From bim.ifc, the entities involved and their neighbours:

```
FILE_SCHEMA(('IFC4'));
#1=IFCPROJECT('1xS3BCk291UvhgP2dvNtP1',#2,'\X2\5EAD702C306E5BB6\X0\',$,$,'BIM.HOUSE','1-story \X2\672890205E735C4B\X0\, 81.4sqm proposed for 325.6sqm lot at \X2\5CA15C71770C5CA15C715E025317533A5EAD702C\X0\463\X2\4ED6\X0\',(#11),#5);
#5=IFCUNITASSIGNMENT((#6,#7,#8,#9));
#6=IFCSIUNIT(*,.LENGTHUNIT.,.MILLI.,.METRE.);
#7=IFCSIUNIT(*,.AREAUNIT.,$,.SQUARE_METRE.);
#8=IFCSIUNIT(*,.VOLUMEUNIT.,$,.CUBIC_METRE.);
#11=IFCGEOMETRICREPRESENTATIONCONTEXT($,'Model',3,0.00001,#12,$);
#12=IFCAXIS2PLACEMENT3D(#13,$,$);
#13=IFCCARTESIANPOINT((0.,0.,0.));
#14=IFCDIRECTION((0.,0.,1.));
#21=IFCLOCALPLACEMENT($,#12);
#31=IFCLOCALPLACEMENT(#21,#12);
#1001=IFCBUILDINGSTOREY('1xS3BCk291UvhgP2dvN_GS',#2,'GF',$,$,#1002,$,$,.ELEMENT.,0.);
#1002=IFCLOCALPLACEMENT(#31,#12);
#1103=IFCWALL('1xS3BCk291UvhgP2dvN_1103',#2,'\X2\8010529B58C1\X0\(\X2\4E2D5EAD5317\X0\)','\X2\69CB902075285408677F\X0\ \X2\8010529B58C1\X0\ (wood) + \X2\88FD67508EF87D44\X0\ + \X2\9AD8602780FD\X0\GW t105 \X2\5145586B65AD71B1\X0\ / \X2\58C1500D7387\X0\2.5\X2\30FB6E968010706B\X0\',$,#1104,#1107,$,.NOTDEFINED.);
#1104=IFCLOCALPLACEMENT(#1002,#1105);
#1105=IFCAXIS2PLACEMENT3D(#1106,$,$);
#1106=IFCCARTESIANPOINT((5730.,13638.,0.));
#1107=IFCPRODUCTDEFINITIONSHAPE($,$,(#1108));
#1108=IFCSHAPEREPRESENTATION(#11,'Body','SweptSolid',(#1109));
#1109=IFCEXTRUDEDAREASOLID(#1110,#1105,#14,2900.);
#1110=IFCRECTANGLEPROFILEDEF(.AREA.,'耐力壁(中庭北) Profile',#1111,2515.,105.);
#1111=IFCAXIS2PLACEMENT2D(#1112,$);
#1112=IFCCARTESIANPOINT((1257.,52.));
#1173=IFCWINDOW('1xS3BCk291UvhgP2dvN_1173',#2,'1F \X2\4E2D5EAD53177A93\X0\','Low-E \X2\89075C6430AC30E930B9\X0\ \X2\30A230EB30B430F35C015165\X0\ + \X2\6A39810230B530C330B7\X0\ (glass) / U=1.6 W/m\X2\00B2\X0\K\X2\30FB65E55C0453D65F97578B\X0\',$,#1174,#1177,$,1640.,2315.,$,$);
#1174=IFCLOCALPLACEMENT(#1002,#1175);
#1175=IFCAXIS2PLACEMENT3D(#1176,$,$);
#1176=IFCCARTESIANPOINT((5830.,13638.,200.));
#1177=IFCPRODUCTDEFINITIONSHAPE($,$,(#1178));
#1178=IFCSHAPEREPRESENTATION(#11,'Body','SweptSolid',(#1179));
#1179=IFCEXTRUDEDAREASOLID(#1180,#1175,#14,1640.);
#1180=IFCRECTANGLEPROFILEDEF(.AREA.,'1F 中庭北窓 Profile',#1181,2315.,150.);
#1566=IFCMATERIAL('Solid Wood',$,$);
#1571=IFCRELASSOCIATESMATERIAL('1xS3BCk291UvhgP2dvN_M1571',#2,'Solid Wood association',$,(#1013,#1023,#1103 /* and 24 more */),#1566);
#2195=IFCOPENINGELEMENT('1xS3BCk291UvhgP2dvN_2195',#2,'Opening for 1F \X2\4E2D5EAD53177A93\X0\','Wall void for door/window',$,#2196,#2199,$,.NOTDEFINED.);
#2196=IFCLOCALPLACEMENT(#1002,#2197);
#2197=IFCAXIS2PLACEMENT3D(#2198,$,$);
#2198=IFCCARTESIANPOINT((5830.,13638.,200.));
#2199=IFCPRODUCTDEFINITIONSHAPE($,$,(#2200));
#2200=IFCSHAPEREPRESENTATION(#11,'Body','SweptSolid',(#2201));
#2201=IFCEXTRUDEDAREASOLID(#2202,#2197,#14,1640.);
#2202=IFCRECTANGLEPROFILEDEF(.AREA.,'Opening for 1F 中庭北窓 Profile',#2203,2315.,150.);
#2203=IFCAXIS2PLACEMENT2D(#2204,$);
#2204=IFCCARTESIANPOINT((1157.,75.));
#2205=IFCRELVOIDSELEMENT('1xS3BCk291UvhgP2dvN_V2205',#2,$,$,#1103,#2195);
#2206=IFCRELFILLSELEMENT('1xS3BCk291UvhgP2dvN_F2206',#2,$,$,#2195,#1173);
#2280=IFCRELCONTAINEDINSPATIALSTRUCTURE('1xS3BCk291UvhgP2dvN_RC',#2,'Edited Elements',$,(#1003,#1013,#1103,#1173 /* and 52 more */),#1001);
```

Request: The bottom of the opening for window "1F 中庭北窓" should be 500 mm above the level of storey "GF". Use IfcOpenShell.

```python
import numpy as np
import ifcopenshell
import ifcopenshell.api.geometry
import ifcopenshell.geom
import ifcopenshell.util.element
import ifcopenshell.util.placement
import ifcopenshell.util.shape
import ifcopenshell.util.unit

model = ifcopenshell.open("bim.ifc")
unit_scale = ifcopenshell.util.unit.calculate_unit_scale(model)

window = model.by_id(1173)
opening = window.FillsVoids[0].RelatingOpeningElement
storey = ifcopenshell.util.element.get_container(window, ifc_class="IfcBuildingStorey")
level = ifcopenshell.util.placement.get_local_placement(storey.ObjectPlacement)[2, 3]

# The opening's origin need not be at the sill, so measure its lowest point.
shape = ifcopenshell.geom.create_shape(ifcopenshell.geom.settings(), opening)
bottom = ifcopenshell.util.shape.get_shape_bottom_elevation(shape, shape.geometry) / unit_scale
dz = level + 500.0 - bottom

shift = np.array([0.0, 0.0, dz])
# The window is not placed relative to its opening, so move both.
for product in (opening, window):
    matrix = ifcopenshell.util.placement.get_local_placement(product.ObjectPlacement)
    matrix[:3, 3] += shift
    ifcopenshell.api.geometry.edit_object_placement(model, product=product, matrix=matrix, is_si=False)

print(f"moved by {dz * unit_scale:+.3f} m")

model.write("bim_v2.ifc")
```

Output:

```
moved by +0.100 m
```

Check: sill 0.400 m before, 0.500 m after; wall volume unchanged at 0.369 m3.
